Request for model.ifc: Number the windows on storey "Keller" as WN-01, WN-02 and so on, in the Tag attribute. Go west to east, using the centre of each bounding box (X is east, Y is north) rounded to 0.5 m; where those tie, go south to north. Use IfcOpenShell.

First a look at what the model holds.

```python
import ifcopenshell
import ifcopenshell.util.element
import ifcopenshell.util.placement

model = ifcopenshell.open("model.ifc")
print(model.schema)
storey = next(s for s in model.by_type("IfcBuildingStorey") if s.Name == "Keller")
windows = [e for e in ifcopenshell.util.element.get_decomposition(storey) if e.is_a("IfcWindow")]
for e in sorted(windows, key=lambda e: e.id()):
    origin = ifcopenshell.util.placement.get_local_placement(e.ObjectPlacement)[:3, 3]
    print(e.id(), e.Tag, e.Name, origin.round(2) + 0.0, sep=" | ")
```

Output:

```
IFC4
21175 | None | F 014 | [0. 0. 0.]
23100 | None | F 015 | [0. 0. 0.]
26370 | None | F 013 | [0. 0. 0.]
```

```python
import ifcopenshell
import ifcopenshell.geom
import ifcopenshell.util.element
import ifcopenshell.util.shape

model = ifcopenshell.open("model.ifc")
settings = ifcopenshell.geom.settings()
settings.set("use-world-coords", True)


def centre(element):
    shape = ifcopenshell.geom.create_shape(settings, element)
    return ifcopenshell.util.shape.get_bbox_centroid(shape.geometry)


storey = next(s for s in model.by_type("IfcBuildingStorey") if s.Name == "Keller")
windows = [e for e in ifcopenshell.util.element.get_decomposition(storey) if e.is_a("IfcWindow")]

# Insertion points can sit at a corner or the storey origin, so sort by the geometry (in metres).
centres = {e: centre(e) for e in windows}
windows.sort(key=lambda e: (round(centres[e][0] / 0.5), centres[e][1]))

for i, e in enumerate(windows, start=1):
    number = f"WN-{i:02d}"
    e.Tag = number
    print(e.id(), number)

model.write("model_v2.ifc")
```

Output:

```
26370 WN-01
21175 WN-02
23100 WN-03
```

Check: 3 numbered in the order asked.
